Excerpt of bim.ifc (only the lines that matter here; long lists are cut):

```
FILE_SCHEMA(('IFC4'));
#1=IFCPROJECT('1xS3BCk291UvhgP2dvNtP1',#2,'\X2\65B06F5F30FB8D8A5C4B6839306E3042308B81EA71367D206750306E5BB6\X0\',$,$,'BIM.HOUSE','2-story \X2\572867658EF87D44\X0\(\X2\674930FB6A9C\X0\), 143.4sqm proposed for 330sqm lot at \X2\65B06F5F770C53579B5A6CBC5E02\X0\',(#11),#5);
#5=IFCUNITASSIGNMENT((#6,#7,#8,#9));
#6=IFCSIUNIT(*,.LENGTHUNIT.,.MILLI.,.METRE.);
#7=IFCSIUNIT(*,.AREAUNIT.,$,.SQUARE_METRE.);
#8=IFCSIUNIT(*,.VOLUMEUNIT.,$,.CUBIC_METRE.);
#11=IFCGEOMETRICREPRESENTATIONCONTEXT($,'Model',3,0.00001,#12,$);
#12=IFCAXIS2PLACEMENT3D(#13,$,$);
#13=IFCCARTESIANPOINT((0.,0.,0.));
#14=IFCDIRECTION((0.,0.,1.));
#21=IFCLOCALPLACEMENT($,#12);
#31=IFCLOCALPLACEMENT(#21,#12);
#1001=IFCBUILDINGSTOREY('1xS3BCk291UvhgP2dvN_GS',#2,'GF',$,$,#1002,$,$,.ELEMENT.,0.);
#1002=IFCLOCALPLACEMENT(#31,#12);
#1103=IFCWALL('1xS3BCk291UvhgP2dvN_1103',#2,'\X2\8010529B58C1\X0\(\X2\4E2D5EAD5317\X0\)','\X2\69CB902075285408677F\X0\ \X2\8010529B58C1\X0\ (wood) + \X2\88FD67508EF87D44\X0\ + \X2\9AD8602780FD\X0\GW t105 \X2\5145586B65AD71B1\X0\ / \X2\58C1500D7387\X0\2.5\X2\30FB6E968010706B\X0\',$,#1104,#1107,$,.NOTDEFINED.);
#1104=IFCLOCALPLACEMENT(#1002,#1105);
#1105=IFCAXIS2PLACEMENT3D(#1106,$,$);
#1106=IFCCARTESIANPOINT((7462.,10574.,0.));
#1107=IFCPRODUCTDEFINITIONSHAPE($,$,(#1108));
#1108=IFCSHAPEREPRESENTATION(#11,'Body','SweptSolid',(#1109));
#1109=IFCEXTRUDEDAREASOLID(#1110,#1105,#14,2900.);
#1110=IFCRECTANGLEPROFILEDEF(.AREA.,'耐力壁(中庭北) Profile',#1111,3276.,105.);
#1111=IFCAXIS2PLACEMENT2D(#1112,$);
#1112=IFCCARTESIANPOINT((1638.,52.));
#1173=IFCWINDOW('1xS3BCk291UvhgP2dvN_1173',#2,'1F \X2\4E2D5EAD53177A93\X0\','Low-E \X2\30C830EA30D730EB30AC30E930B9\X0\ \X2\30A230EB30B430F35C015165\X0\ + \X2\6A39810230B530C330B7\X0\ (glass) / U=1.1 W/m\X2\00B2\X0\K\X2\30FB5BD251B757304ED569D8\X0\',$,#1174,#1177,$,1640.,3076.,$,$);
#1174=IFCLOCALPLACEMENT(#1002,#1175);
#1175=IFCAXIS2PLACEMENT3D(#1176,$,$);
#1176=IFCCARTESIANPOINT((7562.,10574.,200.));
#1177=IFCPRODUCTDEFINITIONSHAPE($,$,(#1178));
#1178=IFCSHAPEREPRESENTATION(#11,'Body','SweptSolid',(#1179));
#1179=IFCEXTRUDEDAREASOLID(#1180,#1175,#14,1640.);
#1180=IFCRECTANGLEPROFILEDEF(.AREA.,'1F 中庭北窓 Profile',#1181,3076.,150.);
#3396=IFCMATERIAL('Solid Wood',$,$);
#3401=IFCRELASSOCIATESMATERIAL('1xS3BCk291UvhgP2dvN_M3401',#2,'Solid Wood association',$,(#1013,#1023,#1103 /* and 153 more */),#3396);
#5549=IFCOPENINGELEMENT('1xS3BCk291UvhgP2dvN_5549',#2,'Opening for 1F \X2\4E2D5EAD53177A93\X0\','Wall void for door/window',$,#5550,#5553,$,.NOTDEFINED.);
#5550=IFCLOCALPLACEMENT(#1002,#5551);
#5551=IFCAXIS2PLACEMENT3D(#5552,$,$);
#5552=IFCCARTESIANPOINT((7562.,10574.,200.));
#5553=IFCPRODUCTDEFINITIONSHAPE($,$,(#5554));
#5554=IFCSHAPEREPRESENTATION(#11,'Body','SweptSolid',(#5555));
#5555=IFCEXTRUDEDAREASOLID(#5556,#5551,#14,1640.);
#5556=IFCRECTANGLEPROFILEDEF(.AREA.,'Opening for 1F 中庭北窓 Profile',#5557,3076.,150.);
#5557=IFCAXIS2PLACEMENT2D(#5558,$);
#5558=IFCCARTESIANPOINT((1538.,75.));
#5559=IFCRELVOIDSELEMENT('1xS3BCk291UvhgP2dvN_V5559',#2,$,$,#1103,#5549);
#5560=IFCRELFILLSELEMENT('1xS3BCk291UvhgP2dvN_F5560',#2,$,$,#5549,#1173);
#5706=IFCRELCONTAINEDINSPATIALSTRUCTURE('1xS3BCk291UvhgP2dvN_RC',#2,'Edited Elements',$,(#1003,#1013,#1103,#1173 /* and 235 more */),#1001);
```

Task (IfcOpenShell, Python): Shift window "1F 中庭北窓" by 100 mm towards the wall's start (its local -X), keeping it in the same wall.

```python
import ifcopenshell
import ifcopenshell.api.geometry
import ifcopenshell.util.placement

model = ifcopenshell.open("bim.ifc")

window = model.by_guid("1xS3BCk291UvhgP2dvN_1173")
opening = window.FillsVoids[0].RelatingOpeningElement
wall = opening.VoidsElements[0].RelatingBuildingElement

wall_matrix = ifcopenshell.util.placement.get_local_placement(wall.ObjectPlacement)
shift = wall_matrix[:3, 0] * -100.0
before = ifcopenshell.util.placement.get_local_placement(window.ObjectPlacement)[:3, 3].copy()

# The window is not placed relative to its opening, so move both.
for product in (opening, window):
    matrix = ifcopenshell.util.placement.get_local_placement(product.ObjectPlacement)
    matrix[:3, 3] += shift
    ifcopenshell.api.geometry.edit_object_placement(model, product=product, matrix=matrix, is_si=False)

after = ifcopenshell.util.placement.get_local_placement(window.ObjectPlacement)[:3, 3]
print("window moved by", (after - before).round(3) + 0.0)

model.write("bim-out.ifc")
```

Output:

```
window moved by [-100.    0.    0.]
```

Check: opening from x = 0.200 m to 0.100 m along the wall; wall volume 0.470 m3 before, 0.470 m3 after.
